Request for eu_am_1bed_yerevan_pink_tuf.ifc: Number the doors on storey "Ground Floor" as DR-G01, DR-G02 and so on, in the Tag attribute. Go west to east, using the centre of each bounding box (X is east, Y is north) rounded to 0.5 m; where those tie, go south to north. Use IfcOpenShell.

First a look at what the model holds.

```python
import ifcopenshell
import ifcopenshell.util.element
import ifcopenshell.util.placement

model = ifcopenshell.open("eu_am_1bed_yerevan_pink_tuf.ifc")
print(model.schema)
storey = next(s for s in model.by_type("IfcBuildingStorey") if s.Name == "Ground Floor")
doors = [e for e in ifcopenshell.util.element.get_decomposition(storey) if e.is_a("IfcDoor")]
for e in sorted(doors, key=lambda e: e.id()):
    origin = ifcopenshell.util.placement.get_local_placement(e.ObjectPlacement)[:3, 3]
    print(e.id(), e.Tag, e.Name, origin.round(2) + 0.0, sep=" | ")
```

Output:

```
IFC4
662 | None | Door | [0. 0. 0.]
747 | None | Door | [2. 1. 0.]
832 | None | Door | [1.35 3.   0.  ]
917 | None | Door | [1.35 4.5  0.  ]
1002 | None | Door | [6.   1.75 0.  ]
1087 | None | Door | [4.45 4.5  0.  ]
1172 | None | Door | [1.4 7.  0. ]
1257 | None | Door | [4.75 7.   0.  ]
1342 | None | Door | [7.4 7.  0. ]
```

```python
import ifcopenshell
import ifcopenshell.geom
import ifcopenshell.util.element
import ifcopenshell.util.shape

model = ifcopenshell.open("eu_am_1bed_yerevan_pink_tuf.ifc")
settings = ifcopenshell.geom.settings()
settings.set("use-world-coords", True)


def centre(element):
    shape = ifcopenshell.geom.create_shape(settings, element)
    return ifcopenshell.util.shape.get_bbox_centroid(shape.geometry)


storey = next(s for s in model.by_type("IfcBuildingStorey") if s.Name == "Ground Floor")
doors = [e for e in ifcopenshell.util.element.get_decomposition(storey) if e.is_a("IfcDoor")]

# Insertion points can sit at a corner or the storey origin, so sort by the geometry (in metres).
centres = {e: centre(e) for e in doors}
doors.sort(key=lambda e: (round(centres[e][0] / 0.5), centres[e][1]))

for i, e in enumerate(doors, start=1):
    number = f"DR-G{i:02d}"
    e.Tag = number
    print(e.id(), number)

model.write("eu_am_1bed_yerevan_pink_tuf-out.ifc")
```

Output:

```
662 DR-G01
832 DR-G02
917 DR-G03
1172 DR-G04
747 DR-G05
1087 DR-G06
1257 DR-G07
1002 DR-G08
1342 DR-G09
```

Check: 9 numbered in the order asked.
